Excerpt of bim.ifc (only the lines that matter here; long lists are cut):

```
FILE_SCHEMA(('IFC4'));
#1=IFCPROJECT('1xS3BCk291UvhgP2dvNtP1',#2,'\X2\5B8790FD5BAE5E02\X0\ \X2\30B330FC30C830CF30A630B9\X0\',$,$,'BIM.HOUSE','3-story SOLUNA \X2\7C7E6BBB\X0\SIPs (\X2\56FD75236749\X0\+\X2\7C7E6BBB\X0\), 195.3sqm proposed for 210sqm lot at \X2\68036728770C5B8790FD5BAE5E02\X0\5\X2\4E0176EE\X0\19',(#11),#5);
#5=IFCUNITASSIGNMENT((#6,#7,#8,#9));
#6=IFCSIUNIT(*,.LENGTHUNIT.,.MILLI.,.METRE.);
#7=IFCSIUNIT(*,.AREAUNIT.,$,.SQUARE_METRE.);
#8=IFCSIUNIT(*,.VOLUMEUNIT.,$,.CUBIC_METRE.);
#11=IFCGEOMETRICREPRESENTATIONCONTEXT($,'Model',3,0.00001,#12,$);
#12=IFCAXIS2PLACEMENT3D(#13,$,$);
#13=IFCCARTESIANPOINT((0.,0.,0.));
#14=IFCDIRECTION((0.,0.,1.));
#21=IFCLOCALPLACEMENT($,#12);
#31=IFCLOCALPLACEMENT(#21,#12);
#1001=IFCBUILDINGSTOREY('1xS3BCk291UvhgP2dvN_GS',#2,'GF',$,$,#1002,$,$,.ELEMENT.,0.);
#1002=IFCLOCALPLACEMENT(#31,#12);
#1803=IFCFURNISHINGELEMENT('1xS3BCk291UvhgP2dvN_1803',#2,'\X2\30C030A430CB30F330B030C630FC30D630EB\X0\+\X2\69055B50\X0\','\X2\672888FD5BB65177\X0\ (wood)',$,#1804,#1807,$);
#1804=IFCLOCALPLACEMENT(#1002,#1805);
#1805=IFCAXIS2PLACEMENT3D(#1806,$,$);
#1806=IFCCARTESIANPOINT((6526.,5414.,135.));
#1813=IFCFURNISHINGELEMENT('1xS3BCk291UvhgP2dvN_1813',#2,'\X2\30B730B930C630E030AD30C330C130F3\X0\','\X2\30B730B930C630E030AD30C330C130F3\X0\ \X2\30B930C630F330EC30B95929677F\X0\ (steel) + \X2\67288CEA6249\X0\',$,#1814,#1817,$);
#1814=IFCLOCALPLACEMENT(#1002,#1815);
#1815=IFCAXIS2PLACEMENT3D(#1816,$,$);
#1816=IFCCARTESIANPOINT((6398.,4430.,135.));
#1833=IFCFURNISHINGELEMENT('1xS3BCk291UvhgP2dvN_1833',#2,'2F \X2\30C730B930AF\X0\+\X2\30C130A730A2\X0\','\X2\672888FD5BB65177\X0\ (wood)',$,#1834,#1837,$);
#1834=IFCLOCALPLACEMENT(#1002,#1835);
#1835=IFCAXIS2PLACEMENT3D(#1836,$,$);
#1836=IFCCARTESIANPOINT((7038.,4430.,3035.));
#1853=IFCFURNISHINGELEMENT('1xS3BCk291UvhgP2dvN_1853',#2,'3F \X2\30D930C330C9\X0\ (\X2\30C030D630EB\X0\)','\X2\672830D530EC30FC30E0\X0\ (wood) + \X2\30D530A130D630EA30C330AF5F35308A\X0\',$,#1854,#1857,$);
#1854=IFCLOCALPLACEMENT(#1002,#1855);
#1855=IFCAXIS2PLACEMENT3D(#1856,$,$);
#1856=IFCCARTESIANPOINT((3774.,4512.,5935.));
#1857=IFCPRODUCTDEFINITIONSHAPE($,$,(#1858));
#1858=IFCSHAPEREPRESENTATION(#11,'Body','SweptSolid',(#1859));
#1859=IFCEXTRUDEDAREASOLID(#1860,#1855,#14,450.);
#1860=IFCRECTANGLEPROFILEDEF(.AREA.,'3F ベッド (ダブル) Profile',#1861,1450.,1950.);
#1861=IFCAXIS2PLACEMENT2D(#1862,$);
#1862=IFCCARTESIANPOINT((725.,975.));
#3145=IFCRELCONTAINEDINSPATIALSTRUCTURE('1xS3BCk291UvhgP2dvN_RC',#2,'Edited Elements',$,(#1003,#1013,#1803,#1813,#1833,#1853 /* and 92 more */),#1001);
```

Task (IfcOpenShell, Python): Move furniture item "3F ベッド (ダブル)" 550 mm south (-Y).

```python
import ifcopenshell
import ifcopenshell.api.geometry
import ifcopenshell.util.placement

model = ifcopenshell.open("bim.ifc")

item = model.by_guid("1xS3BCk291UvhgP2dvN_1853")
matrix = ifcopenshell.util.placement.get_local_placement(item.ObjectPlacement)
matrix[1, 3] -= 550.0
ifcopenshell.api.geometry.edit_object_placement(model, product=item, matrix=matrix, is_si=False)

print(ifcopenshell.util.placement.get_local_placement(item.ObjectPlacement).round(3) + 0.0)

model.write("bim_edited.ifc")
```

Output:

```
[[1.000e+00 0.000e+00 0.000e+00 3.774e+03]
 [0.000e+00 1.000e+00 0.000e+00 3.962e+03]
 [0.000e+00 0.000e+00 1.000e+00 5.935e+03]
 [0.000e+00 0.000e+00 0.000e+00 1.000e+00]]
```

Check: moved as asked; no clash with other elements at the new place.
